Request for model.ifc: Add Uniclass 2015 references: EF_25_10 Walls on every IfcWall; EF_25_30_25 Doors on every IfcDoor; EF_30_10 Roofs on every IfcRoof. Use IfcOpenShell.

First a look at what the model holds.

```python
import ifcopenshell

model = ifcopenshell.open("model.ifc")
print(model.schema)
print("classifications:", [c.Name for c in model.by_type("IfcClassification")])
for ifc_class in ("IfcDoor", "IfcRoof", "IfcStair", "IfcWall", "IfcWindow"):
    print(ifc_class, len(model.by_type(ifc_class)))
```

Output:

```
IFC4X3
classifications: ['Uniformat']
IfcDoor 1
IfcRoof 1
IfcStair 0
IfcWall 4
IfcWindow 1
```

```python
import ifcopenshell
import ifcopenshell.api.classification

model = ifcopenshell.open("model.ifc")

system = ifcopenshell.api.classification.add_classification(model, classification="Uniclass 2015")

codes = {
    "IfcWall": ("EF_25_10", "Walls"),
    "IfcDoor": ("EF_25_30_25", "Doors"),
    "IfcRoof": ("EF_30_10", "Roofs"),
}
for ifc_class, (code, name) in codes.items():
    products = model.by_type(ifc_class)
    ifcopenshell.api.classification.add_reference(
        model, products=products, classification=system, identification=code, name=name
    )
    print(code, len(products))

model.write("model_v2.ifc")
```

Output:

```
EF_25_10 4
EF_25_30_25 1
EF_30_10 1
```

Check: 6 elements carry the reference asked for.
